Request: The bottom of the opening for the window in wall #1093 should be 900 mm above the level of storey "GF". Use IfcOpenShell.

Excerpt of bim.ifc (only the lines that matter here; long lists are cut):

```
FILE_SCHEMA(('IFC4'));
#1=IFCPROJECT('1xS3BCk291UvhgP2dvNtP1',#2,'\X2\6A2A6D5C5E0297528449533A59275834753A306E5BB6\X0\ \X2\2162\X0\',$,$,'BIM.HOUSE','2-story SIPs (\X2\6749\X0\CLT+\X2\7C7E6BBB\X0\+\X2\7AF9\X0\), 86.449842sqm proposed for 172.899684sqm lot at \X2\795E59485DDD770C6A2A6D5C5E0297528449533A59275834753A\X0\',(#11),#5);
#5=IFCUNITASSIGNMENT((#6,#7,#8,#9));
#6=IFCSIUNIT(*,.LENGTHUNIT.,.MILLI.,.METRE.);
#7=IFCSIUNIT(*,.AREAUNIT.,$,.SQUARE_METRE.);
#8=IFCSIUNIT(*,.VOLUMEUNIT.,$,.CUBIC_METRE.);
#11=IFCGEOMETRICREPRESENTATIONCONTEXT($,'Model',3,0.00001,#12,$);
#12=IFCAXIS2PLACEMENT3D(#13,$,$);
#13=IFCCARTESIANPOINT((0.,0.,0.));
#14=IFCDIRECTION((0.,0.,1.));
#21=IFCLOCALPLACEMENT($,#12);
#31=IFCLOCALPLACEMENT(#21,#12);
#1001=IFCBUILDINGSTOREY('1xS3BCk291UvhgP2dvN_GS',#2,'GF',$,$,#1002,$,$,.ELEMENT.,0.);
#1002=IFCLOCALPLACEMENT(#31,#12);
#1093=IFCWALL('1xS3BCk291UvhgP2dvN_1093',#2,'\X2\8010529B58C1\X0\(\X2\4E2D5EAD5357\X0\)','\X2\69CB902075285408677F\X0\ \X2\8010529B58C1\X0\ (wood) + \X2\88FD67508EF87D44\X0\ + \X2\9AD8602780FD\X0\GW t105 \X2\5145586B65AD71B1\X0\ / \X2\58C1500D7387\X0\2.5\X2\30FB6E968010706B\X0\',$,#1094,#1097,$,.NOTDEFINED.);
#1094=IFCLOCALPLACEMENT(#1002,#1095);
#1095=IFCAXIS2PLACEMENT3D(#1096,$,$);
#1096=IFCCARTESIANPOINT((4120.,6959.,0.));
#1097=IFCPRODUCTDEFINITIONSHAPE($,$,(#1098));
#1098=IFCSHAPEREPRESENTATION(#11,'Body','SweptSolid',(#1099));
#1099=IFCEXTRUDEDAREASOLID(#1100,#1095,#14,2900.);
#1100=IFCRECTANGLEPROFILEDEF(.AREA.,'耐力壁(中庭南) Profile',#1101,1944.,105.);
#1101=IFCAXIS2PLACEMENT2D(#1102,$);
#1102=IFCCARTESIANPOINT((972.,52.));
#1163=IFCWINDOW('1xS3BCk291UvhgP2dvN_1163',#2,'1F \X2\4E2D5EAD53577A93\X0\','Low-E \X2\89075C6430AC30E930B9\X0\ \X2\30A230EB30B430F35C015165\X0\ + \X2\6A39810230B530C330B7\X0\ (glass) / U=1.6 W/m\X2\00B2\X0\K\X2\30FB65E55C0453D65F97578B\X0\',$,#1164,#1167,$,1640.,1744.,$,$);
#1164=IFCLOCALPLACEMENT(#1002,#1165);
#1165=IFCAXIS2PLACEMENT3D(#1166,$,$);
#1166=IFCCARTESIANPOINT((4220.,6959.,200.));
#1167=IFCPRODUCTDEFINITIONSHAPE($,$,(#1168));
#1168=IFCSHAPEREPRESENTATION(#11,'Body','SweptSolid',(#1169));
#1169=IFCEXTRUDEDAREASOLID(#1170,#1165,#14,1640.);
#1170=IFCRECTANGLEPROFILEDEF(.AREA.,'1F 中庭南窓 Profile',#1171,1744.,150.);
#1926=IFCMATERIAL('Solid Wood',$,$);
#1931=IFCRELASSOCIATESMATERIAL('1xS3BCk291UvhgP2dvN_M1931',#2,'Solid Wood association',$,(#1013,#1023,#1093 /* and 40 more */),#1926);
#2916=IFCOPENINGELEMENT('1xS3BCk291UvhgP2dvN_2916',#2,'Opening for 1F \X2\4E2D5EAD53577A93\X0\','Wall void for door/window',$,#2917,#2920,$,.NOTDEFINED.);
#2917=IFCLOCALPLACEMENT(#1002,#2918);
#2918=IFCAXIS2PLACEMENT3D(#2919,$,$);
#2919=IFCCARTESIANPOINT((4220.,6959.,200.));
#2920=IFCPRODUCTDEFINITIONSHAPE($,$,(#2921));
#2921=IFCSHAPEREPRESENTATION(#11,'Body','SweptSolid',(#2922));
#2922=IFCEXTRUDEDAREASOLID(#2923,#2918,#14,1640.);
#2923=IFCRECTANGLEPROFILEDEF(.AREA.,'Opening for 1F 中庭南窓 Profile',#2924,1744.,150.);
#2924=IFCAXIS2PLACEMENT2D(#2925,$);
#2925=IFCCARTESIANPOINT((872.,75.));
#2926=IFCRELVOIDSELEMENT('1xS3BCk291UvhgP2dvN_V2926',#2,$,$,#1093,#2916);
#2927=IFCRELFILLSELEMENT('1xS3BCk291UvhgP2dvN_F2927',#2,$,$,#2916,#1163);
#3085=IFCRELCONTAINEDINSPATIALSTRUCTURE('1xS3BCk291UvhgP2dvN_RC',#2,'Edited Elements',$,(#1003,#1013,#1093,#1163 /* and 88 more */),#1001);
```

```python
import numpy as np
import ifcopenshell
import ifcopenshell.api.geometry
import ifcopenshell.geom
import ifcopenshell.util.element
import ifcopenshell.util.placement
import ifcopenshell.util.shape
import ifcopenshell.util.unit

model = ifcopenshell.open("bim.ifc")
unit_scale = ifcopenshell.util.unit.calculate_unit_scale(model)

window = model.by_guid("1xS3BCk291UvhgP2dvN_1163")
opening = window.FillsVoids[0].RelatingOpeningElement
storey = ifcopenshell.util.element.get_container(window, ifc_class="IfcBuildingStorey")
level = ifcopenshell.util.placement.get_local_placement(storey.ObjectPlacement)[2, 3]

# The opening's origin need not be at the sill, so measure its lowest point.
shape = ifcopenshell.geom.create_shape(ifcopenshell.geom.settings(), opening)
bottom = ifcopenshell.util.shape.get_shape_bottom_elevation(shape, shape.geometry) / unit_scale
dz = level + 900.0 - bottom

shift = np.array([0.0, 0.0, dz])
# The window is not placed relative to its opening, so move both.
for product in (opening, window):
    matrix = ifcopenshell.util.placement.get_local_placement(product.ObjectPlacement)
    matrix[:3, 3] += shift
    ifcopenshell.api.geometry.edit_object_placement(model, product=product, matrix=matrix, is_si=False)

print(f"moved by {dz * unit_scale:+.3f} m")

model.write("bim_edited.ifc")
```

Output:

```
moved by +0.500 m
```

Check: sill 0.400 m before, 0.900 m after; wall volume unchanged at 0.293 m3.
